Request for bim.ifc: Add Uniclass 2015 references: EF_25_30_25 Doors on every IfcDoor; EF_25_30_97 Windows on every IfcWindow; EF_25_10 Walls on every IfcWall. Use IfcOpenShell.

First a look at what the model holds.

```python
import ifcopenshell

model = ifcopenshell.open("bim.ifc")
print(model.schema)
print("classifications:", [c.Name for c in model.by_type("IfcClassification")])
for ifc_class in ("IfcDoor", "IfcRoof", "IfcStair", "IfcWall", "IfcWindow"):
    print(ifc_class, len(model.by_type(ifc_class)))
```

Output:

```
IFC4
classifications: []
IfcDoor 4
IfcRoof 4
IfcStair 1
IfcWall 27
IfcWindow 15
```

```python
import ifcopenshell
import ifcopenshell.api.classification

model = ifcopenshell.open("bim.ifc")

system = ifcopenshell.api.classification.add_classification(model, classification="Uniclass 2015")

codes = {
    "IfcDoor": ("EF_25_30_25", "Doors"),
    "IfcWindow": ("EF_25_30_97", "Windows"),
    "IfcWall": ("EF_25_10", "Walls"),
}
for ifc_class, (code, name) in codes.items():
    products = model.by_type(ifc_class)
    ifcopenshell.api.classification.add_reference(
        model, products=products, classification=system, identification=code, name=name
    )
    print(code, len(products))

model.write("bim-out.ifc")
```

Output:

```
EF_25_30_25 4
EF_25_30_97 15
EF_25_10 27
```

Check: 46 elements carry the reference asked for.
